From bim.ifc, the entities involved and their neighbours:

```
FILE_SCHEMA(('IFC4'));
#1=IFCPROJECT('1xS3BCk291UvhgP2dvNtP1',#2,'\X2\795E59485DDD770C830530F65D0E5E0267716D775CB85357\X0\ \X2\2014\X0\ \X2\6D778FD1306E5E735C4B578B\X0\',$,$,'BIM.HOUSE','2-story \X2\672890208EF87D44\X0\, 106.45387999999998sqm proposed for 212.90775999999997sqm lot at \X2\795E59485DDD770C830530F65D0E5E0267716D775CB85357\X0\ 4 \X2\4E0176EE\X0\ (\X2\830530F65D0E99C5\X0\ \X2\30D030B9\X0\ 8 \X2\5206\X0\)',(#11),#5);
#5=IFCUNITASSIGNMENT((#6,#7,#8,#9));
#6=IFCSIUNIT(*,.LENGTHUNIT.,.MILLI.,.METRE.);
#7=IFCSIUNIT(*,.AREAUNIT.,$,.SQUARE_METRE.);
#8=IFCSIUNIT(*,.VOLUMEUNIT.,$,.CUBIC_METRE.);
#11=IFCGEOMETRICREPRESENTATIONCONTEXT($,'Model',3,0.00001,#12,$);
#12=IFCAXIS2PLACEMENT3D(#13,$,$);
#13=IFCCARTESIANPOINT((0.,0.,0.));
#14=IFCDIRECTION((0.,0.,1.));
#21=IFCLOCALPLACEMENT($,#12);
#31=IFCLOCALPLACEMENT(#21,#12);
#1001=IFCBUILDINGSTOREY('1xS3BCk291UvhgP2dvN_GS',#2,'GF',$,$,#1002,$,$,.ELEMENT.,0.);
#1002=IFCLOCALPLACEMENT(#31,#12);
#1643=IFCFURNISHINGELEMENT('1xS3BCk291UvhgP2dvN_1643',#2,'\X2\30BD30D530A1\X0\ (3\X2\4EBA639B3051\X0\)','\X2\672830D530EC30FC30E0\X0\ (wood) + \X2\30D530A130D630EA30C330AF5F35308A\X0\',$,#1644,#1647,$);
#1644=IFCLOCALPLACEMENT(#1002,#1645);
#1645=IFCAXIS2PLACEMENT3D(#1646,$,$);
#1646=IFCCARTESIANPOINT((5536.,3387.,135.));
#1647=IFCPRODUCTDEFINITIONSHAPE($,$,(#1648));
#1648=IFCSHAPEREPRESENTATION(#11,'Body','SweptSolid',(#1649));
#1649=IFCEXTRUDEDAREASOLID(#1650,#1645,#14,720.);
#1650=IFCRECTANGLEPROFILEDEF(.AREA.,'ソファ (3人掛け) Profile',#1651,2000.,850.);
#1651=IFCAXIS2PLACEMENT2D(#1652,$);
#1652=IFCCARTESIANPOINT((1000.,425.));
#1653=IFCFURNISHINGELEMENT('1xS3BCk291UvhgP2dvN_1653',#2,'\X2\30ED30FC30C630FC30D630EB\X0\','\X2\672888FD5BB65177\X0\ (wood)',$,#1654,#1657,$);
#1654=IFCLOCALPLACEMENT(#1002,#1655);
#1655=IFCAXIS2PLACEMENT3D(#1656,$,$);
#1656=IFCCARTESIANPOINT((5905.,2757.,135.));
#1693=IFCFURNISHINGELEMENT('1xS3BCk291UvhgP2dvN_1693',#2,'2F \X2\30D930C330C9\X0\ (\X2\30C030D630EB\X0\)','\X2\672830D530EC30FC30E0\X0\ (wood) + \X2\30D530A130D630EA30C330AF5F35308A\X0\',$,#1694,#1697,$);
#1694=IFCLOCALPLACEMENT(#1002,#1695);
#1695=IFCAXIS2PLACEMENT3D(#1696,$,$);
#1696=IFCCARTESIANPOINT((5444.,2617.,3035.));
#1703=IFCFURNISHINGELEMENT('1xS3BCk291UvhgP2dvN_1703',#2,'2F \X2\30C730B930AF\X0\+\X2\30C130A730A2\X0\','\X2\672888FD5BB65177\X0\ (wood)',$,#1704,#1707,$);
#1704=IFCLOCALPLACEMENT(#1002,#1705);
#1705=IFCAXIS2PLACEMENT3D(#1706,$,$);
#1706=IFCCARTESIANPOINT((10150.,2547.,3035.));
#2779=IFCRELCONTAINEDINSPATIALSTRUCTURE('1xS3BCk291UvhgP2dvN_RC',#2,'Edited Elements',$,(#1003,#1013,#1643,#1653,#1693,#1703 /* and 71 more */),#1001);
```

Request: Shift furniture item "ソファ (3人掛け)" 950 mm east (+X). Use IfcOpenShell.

```python
import ifcopenshell
import ifcopenshell.api.geometry
import ifcopenshell.util.placement

model = ifcopenshell.open("bim.ifc")

item = model.by_id(1643)
matrix = ifcopenshell.util.placement.get_local_placement(item.ObjectPlacement)
matrix[0, 3] += 950.0
ifcopenshell.api.geometry.edit_object_placement(model, product=item, matrix=matrix, is_si=False)

print(ifcopenshell.util.placement.get_local_placement(item.ObjectPlacement).round(3) + 0.0)

model.write("bim_rev.ifc")
```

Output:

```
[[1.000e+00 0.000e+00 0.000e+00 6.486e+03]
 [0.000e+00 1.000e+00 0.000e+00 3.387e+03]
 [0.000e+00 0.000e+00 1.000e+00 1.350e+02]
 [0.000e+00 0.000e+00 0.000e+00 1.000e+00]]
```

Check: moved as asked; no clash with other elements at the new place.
